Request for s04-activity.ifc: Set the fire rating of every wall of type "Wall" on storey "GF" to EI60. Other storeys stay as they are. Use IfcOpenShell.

First a look at what the model holds.

```python
import ifcopenshell
import ifcopenshell.util.element

model = ifcopenshell.open("s04-activity.ifc")
print(model.schema)
storey = next(s for s in model.by_type("IfcBuildingStorey") if s.Name == "GF")
walls = [e for e in ifcopenshell.util.element.get_decomposition(storey) if e.is_a("IfcWall")]
seen = {}
for e in walls:
    element_type = ifcopenshell.util.element.get_type(e)
    key = (element_type.Name if element_type != e and element_type else None, ifcopenshell.util.element.get_pset(e, "Pset_WallCommon", "FireRating"))
    seen[key] = seen.get(key, 0) + 1
for (name, value), count in sorted(seen.items(), key=str):
    print(count, "x", name, "|", value)
```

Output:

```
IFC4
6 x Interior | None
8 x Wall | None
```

```python
import ifcopenshell
import ifcopenshell.api.pset
import ifcopenshell.util.element

model = ifcopenshell.open("s04-activity.ifc")

storey = next(s for s in model.by_type("IfcBuildingStorey") if s.Name == "GF")
walls = [e for e in ifcopenshell.util.element.get_decomposition(storey) if e.is_a("IfcWall")]

count = 0
for e in walls:
    element_type = ifcopenshell.util.element.get_type(e)
    if element_type in (None, e) or element_type.Name != "Wall":
        continue
    # add_pset returns the element's existing set when there is one.
    pset = ifcopenshell.api.pset.add_pset(model, product=e, name="Pset_WallCommon")
    ifcopenshell.api.pset.edit_pset(model, pset=pset, properties={"FireRating": "EI60"})
    count += 1

print(count, "walls updated")

model.write("s04-activity_v2.ifc")
```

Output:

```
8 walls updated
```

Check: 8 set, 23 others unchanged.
